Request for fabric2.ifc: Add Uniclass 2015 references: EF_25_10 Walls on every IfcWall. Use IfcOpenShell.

First a look at what the model holds.

```python
import ifcopenshell

model = ifcopenshell.open("fabric2.ifc")
print(model.schema)
print("classifications:", [c.Name for c in model.by_type("IfcClassification")])
for ifc_class in ("IfcDoor", "IfcRoof", "IfcStair", "IfcWall", "IfcWindow"):
    print(ifc_class, len(model.by_type(ifc_class)))
```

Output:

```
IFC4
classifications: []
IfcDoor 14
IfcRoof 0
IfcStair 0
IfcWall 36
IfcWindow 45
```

```python
import ifcopenshell
import ifcopenshell.api.classification

model = ifcopenshell.open("fabric2.ifc")

system = ifcopenshell.api.classification.add_classification(model, classification="Uniclass 2015")

codes = {
    "IfcWall": ("EF_25_10", "Walls"),
}
for ifc_class, (code, name) in codes.items():
    products = model.by_type(ifc_class)
    ifcopenshell.api.classification.add_reference(
        model, products=products, classification=system, identification=code, name=name
    )
    print(code, len(products))

model.write("fabric2_updated.ifc")
```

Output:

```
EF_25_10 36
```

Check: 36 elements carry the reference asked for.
